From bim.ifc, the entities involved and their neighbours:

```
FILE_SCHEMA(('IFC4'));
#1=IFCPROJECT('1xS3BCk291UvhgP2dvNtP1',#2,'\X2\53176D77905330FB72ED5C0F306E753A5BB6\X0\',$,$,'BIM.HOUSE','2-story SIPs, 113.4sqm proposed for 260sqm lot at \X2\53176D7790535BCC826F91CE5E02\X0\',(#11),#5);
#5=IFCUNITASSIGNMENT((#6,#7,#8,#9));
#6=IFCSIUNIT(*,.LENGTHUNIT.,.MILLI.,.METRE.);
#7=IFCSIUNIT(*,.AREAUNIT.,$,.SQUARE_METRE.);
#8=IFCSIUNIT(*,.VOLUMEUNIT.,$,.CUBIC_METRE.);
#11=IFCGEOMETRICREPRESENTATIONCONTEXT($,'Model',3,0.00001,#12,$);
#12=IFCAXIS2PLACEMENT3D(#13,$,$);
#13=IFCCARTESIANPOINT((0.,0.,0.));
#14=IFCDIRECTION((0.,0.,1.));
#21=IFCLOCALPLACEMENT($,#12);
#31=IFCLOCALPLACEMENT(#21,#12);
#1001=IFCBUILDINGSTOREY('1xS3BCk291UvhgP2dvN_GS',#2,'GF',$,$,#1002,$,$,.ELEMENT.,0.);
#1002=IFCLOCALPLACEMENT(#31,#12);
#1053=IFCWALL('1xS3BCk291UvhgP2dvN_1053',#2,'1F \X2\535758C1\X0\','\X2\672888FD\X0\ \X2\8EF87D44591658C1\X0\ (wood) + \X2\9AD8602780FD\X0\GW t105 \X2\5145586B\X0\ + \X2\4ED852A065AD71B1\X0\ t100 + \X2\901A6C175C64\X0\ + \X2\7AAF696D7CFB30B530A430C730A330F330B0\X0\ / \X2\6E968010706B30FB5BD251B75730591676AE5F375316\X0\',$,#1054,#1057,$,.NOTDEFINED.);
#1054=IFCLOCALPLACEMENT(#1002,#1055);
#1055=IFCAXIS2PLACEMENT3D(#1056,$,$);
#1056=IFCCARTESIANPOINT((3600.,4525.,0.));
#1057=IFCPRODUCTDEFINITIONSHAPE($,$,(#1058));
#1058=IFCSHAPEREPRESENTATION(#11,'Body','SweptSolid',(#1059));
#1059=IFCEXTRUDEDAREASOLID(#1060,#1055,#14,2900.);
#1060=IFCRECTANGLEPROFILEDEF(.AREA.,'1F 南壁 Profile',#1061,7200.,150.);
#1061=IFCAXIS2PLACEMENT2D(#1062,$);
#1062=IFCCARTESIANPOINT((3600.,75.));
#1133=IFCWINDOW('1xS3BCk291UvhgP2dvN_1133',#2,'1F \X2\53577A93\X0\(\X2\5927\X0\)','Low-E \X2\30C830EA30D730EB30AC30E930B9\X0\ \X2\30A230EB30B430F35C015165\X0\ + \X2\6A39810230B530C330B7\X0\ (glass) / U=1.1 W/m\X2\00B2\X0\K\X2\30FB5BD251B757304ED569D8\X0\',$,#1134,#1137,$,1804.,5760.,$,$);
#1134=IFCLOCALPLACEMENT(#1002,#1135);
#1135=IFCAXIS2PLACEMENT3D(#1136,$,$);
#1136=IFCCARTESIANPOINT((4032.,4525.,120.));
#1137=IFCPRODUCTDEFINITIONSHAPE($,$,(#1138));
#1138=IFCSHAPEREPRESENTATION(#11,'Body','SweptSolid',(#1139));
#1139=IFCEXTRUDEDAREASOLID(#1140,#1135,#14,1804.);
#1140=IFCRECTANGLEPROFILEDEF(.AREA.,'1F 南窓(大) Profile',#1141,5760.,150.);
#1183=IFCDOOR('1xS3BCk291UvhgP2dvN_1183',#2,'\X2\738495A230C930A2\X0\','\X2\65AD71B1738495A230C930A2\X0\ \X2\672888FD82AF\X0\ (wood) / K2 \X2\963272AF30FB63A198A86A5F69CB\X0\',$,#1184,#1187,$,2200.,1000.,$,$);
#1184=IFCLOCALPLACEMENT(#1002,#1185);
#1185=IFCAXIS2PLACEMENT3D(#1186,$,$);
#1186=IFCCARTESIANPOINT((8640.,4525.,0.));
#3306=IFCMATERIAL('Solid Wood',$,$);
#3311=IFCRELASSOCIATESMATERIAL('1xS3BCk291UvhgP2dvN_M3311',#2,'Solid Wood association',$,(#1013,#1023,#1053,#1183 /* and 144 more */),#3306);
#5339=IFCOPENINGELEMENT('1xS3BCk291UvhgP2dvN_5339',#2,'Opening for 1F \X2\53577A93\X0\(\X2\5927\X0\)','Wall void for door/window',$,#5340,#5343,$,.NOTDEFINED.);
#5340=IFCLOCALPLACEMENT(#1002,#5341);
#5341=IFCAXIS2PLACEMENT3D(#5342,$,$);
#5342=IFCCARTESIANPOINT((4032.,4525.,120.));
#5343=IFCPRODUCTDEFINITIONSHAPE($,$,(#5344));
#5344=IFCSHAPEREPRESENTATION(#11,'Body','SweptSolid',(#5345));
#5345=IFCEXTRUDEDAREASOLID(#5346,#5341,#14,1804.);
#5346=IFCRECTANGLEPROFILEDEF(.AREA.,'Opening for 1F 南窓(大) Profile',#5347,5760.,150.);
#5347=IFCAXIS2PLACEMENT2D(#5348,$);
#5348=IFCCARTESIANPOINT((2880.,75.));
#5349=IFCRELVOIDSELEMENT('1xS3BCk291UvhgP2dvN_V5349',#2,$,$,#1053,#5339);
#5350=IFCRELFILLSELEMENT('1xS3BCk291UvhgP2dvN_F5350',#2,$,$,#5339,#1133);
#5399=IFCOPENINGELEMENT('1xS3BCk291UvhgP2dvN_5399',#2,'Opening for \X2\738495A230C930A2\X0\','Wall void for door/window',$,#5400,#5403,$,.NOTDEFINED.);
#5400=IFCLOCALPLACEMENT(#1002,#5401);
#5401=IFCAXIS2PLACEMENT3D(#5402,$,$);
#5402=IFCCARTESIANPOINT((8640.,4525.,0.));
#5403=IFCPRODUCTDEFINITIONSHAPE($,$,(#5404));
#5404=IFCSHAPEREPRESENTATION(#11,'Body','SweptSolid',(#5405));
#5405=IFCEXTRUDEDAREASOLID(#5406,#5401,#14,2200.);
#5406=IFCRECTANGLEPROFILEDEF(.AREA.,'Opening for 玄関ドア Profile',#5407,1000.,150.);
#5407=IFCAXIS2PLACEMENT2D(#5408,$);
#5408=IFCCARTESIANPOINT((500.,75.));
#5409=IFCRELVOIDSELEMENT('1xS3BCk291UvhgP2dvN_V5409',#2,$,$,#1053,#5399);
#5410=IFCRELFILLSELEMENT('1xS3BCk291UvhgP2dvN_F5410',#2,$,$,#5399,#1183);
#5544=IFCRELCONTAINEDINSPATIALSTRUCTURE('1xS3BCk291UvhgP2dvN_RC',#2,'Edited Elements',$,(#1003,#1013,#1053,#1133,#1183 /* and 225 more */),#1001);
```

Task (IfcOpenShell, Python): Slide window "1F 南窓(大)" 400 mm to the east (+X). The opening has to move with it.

```python
import ifcopenshell
import ifcopenshell.api.geometry
import ifcopenshell.util.placement

model = ifcopenshell.open("bim.ifc")

window = model.by_id(1133)
opening = window.FillsVoids[0].RelatingOpeningElement
wall = opening.VoidsElements[0].RelatingBuildingElement

wall_matrix = ifcopenshell.util.placement.get_local_placement(wall.ObjectPlacement)
shift = wall_matrix[:3, 0] * 400.0
before = ifcopenshell.util.placement.get_local_placement(window.ObjectPlacement)[:3, 3].copy()

# The window is not placed relative to its opening, so move both.
for product in (opening, window):
    matrix = ifcopenshell.util.placement.get_local_placement(product.ObjectPlacement)
    matrix[:3, 3] += shift
    ifcopenshell.api.geometry.edit_object_placement(model, product=product, matrix=matrix, is_si=False)

after = ifcopenshell.util.placement.get_local_placement(window.ObjectPlacement)[:3, 3]
print("window moved by", (after - before).round(3) + 0.0)

model.write("bim_updated.ifc")
```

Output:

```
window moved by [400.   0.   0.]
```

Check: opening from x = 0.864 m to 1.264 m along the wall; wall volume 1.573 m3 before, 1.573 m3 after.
